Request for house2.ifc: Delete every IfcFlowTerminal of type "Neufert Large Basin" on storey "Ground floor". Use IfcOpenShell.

First a look at what the model holds.

```python
import ifcopenshell
import ifcopenshell.util.element

model = ifcopenshell.open("house2.ifc")
print(model.schema)
storey = next(s for s in model.by_type("IfcBuildingStorey") if s.Name == "Ground floor")
terminals = [e for e in ifcopenshell.util.element.get_decomposition(storey) if e.is_a("IfcFlowTerminal")]
seen = {}
for e in terminals:
    element_type = ifcopenshell.util.element.get_type(e)
    name = element_type.Name if element_type not in (None, e) else None
    seen[name] = seen.get(name, 0) + 1
for name, count in sorted(seen.items(), key=str):
    print(count, "x", name)
```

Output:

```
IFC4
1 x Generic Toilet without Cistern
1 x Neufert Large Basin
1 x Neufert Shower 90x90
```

```python
import ifcopenshell
import ifcopenshell.api.root
import ifcopenshell.util.element

model = ifcopenshell.open("house2.ifc")

storey = next(s for s in model.by_type("IfcBuildingStorey") if s.Name == "Ground floor")
terminals = [e for e in ifcopenshell.util.element.get_decomposition(storey) if e.is_a("IfcFlowTerminal")]
targets = [e for e in terminals if (t := ifcopenshell.util.element.get_type(e)) not in (None, e) and t.Name == "Neufert Large Basin"]

for e in targets:
    ifcopenshell.api.root.remove_product(model, product=e)
print(len(targets), "removed")

model.write("house2_v2.ifc")
```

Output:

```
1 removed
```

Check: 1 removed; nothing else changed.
